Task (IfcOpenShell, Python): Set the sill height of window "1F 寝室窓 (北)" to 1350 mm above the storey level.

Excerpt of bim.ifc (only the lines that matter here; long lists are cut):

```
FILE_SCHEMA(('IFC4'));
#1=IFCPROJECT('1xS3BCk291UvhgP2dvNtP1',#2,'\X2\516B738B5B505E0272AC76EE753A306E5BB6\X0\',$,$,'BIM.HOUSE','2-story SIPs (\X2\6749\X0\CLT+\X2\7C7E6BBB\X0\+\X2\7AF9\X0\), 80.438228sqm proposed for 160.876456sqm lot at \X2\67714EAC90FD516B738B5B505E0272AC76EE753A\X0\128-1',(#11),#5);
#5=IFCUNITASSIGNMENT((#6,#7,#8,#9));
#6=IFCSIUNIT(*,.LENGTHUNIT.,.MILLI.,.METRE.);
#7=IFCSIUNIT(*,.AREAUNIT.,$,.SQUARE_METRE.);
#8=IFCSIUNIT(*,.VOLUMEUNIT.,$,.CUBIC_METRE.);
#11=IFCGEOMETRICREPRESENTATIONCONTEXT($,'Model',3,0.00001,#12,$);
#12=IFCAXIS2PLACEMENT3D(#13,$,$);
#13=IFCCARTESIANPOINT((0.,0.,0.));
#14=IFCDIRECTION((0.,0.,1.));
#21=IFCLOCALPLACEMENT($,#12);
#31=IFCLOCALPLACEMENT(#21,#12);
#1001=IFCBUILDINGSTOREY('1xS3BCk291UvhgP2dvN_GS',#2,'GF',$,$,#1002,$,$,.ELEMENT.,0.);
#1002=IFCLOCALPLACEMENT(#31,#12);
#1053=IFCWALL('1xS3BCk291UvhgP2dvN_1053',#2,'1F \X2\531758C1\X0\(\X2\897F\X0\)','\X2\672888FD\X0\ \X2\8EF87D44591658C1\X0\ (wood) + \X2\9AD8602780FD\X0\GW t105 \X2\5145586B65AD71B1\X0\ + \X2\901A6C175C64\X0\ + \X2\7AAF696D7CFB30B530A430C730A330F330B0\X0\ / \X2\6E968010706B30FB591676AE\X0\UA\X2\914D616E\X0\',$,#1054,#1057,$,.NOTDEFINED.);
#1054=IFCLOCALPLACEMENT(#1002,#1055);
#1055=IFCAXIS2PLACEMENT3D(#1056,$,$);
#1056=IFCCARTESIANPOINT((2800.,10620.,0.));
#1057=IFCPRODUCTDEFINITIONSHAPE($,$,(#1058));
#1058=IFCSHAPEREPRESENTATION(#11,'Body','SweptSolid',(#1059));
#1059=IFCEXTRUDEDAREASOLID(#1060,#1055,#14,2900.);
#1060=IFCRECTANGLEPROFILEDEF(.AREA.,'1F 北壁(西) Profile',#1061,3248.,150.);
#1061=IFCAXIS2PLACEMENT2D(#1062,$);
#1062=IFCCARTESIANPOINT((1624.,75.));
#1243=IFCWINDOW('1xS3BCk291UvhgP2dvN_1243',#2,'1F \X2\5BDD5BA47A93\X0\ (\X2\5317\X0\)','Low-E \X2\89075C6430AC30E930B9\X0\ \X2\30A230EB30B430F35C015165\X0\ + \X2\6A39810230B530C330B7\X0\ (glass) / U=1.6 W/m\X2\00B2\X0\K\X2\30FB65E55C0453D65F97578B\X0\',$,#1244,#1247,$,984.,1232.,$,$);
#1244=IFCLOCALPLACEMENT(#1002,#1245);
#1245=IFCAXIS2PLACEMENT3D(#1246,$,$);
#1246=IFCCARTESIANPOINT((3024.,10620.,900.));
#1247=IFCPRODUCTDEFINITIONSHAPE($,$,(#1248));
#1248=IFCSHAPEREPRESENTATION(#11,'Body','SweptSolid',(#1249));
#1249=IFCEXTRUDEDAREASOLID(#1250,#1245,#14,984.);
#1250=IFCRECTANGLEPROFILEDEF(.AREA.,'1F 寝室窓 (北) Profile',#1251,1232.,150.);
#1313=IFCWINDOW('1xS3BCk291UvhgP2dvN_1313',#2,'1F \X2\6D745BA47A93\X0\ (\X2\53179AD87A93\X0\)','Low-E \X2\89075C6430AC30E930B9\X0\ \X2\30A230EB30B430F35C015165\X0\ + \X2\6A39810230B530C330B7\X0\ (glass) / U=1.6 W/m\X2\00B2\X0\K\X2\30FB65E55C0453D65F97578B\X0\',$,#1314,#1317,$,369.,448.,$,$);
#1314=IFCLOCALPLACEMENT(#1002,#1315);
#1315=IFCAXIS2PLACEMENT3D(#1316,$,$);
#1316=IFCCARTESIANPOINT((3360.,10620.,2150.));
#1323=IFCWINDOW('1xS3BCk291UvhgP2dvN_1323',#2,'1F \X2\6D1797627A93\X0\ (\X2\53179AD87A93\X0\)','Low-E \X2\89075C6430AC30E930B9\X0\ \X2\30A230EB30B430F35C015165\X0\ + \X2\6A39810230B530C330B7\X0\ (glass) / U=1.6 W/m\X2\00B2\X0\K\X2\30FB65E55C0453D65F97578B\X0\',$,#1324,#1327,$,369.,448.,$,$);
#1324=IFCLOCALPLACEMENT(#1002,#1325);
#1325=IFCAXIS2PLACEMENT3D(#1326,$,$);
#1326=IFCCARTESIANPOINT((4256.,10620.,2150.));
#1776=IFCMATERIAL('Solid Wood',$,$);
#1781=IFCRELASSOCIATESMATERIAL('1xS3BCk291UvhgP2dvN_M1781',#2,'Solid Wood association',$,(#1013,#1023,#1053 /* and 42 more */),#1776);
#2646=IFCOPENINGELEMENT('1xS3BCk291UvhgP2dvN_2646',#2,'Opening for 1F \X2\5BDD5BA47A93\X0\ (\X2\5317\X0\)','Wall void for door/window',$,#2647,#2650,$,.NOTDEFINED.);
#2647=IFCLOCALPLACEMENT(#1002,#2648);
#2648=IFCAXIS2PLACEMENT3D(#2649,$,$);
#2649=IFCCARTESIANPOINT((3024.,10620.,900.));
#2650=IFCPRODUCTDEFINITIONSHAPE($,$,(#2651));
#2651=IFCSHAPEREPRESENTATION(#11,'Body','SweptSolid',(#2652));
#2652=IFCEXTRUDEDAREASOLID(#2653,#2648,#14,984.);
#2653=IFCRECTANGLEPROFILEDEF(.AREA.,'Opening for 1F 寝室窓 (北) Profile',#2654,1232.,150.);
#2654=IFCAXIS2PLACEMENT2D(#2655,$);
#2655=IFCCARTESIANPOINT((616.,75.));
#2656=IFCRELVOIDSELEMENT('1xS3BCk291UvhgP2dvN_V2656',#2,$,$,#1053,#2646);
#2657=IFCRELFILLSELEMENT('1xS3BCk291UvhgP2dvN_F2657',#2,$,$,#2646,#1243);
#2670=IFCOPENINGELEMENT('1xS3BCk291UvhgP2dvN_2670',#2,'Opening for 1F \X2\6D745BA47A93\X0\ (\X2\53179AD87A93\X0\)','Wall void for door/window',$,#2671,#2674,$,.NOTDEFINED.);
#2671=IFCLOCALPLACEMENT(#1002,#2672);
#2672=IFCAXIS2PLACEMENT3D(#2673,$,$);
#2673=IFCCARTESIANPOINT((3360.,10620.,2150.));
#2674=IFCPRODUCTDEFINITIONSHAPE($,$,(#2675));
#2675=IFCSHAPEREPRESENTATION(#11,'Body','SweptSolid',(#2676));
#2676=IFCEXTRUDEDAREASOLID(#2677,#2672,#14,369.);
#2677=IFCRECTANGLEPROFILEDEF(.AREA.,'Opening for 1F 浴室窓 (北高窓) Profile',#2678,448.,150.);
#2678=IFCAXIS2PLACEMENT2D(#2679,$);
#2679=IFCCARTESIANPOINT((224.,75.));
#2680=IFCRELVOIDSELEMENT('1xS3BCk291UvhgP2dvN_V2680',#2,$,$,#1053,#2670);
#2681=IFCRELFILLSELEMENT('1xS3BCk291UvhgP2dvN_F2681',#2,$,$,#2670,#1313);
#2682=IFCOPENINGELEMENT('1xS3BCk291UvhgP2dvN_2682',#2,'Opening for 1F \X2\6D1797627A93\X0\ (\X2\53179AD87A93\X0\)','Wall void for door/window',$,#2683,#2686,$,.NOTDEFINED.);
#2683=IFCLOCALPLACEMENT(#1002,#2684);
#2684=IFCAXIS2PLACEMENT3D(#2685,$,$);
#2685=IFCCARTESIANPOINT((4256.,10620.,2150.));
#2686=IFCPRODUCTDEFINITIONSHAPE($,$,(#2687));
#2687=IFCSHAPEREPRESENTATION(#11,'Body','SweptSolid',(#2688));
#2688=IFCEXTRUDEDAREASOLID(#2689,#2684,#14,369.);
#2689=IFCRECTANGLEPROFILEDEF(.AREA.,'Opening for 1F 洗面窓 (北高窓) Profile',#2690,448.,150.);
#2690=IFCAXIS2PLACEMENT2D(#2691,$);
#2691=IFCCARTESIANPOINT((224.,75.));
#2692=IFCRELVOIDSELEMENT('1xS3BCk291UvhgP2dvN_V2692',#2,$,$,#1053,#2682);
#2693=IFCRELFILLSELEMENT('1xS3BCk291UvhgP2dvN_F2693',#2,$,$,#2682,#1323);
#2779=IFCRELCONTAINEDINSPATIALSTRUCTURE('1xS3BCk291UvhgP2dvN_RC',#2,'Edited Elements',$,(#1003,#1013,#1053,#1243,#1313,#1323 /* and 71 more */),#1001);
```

```python
import numpy as np
import ifcopenshell
import ifcopenshell.api.geometry
import ifcopenshell.geom
import ifcopenshell.util.element
import ifcopenshell.util.placement
import ifcopenshell.util.shape
import ifcopenshell.util.unit

model = ifcopenshell.open("bim.ifc")
unit_scale = ifcopenshell.util.unit.calculate_unit_scale(model)

window = model.by_guid("1xS3BCk291UvhgP2dvN_1243")
opening = window.FillsVoids[0].RelatingOpeningElement
storey = ifcopenshell.util.element.get_container(window, ifc_class="IfcBuildingStorey")
level = ifcopenshell.util.placement.get_local_placement(storey.ObjectPlacement)[2, 3]

# The opening's origin need not be at the sill, so measure its lowest point.
shape = ifcopenshell.geom.create_shape(ifcopenshell.geom.settings(), opening)
bottom = ifcopenshell.util.shape.get_shape_bottom_elevation(shape, shape.geometry) / unit_scale
dz = level + 1350.0 - bottom

shift = np.array([0.0, 0.0, dz])
# The window is not placed relative to its opening, so move both.
for product in (opening, window):
    matrix = ifcopenshell.util.placement.get_local_placement(product.ObjectPlacement)
    matrix[:3, 3] += shift
    ifcopenshell.api.geometry.edit_object_placement(model, product=product, matrix=matrix, is_si=False)

print(f"moved by {dz * unit_scale:+.3f} m")

model.write("bim-out.ifc")
```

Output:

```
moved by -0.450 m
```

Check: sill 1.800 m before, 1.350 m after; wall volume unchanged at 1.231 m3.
